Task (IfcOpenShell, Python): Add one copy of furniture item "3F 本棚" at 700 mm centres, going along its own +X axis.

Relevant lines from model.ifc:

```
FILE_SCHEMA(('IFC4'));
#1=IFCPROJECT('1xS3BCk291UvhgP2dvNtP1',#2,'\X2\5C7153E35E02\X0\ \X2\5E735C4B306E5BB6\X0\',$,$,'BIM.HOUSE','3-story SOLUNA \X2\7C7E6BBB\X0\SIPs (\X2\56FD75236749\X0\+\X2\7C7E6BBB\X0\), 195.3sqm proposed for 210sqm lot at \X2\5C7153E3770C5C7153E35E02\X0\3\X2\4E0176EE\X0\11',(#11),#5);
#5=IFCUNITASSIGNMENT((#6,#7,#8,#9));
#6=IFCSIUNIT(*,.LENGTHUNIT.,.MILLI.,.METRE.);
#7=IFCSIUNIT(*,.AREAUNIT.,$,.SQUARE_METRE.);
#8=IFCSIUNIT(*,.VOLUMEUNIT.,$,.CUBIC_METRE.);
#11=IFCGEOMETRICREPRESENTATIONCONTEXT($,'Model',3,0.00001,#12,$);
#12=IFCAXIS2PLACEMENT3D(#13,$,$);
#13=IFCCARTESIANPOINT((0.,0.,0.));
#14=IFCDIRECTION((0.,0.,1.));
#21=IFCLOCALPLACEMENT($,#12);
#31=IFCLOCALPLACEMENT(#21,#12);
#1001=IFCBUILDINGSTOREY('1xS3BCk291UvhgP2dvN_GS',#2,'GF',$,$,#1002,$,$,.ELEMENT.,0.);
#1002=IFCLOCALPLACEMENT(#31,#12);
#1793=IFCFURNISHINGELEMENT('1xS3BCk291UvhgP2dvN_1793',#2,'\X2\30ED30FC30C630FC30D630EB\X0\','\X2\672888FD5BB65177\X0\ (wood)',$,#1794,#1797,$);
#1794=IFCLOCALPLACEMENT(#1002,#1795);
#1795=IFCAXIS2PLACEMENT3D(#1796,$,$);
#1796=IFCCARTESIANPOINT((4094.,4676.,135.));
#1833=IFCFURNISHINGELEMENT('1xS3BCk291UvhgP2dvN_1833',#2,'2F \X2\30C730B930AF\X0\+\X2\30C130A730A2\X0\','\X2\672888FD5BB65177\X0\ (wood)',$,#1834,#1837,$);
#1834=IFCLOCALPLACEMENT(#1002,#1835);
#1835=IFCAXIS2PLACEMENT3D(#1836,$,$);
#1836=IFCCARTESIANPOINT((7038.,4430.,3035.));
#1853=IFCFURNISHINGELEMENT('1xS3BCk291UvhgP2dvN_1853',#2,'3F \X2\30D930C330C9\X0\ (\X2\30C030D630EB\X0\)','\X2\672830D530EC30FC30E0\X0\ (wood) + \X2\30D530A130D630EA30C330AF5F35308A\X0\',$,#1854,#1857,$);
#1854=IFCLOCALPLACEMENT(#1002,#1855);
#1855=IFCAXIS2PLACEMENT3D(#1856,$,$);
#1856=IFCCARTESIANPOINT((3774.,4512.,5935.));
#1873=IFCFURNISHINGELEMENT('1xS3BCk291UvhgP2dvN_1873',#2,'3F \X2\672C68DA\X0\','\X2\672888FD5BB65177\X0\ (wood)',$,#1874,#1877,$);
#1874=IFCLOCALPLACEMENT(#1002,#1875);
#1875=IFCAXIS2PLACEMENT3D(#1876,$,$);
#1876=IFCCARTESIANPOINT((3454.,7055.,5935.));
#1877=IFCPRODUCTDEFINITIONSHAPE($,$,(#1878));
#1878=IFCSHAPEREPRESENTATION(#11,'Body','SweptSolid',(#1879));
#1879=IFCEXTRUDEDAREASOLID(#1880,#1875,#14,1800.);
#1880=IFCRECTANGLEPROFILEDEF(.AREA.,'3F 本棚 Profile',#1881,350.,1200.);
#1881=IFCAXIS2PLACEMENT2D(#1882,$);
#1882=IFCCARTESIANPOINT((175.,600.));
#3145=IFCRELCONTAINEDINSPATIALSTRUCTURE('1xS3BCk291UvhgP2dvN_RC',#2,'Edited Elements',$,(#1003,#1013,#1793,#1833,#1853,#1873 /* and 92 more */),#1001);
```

```python
import ifcopenshell
import ifcopenshell.api.geometry
import ifcopenshell.api.root
import ifcopenshell.util.element
import ifcopenshell.util.placement
import ifcopenshell.util.unit

model = ifcopenshell.open("model.ifc")
unit_scale = ifcopenshell.util.unit.calculate_unit_scale(model)


def reuse_history(source, copy):
    """copy_class also copies each property set's owner history, people and application; keep the originals."""
    for rel in copy.IsDefinedBy:
        if rel.is_a("IfcRelDefinesByProperties") and (history := rel.RelatingPropertyDefinition.OwnerHistory):
            rel.RelatingPropertyDefinition.OwnerHistory = source.OwnerHistory
            ifcopenshell.util.element.remove_deep2(model, history)


source = model.by_guid("1xS3BCk291UvhgP2dvN_1873")
base = ifcopenshell.util.placement.get_local_placement(source.ObjectPlacement)
step = base[:3, 0] * 0.7 / unit_scale

for i in range(1, 2):
    copy = ifcopenshell.api.root.copy_class(model, product=source)
    copy.Representation = ifcopenshell.util.element.copy_deep(
        model, source.Representation, exclude=["IfcGeometricRepresentationContext", "IfcRepresentationMap"]
    )
    reuse_history(source, copy)
    matrix = base.copy()
    matrix[:3, 3] += i * step
    print("added at", matrix[:3, 3].round(3) + 0.0)
    ifcopenshell.api.geometry.edit_object_placement(model, product=copy, matrix=matrix, is_si=False)

model.write("model-out.ifc")
```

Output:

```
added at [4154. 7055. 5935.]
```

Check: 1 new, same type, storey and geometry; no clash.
